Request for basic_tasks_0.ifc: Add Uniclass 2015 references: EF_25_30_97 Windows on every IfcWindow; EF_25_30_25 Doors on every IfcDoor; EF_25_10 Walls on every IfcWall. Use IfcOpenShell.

First a look at what the model holds.

```python
import ifcopenshell

model = ifcopenshell.open("basic_tasks_0.ifc")
print(model.schema)
print("classifications:", [c.Name for c in model.by_type("IfcClassification")])
for ifc_class in ("IfcDoor", "IfcRoof", "IfcStair", "IfcWall", "IfcWindow"):
    print(ifc_class, len(model.by_type(ifc_class)))
```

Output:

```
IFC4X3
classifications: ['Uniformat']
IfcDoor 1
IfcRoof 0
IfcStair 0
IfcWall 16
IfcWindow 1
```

```python
import ifcopenshell
import ifcopenshell.api.classification

model = ifcopenshell.open("basic_tasks_0.ifc")

system = ifcopenshell.api.classification.add_classification(model, classification="Uniclass 2015")

codes = {
    "IfcWindow": ("EF_25_30_97", "Windows"),
    "IfcDoor": ("EF_25_30_25", "Doors"),
    "IfcWall": ("EF_25_10", "Walls"),
}
for ifc_class, (code, name) in codes.items():
    products = model.by_type(ifc_class)
    ifcopenshell.api.classification.add_reference(
        model, products=products, classification=system, identification=code, name=name
    )
    print(code, len(products))

model.write("basic_tasks_0-out.ifc")
```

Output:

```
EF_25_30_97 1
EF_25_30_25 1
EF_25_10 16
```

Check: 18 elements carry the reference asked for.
